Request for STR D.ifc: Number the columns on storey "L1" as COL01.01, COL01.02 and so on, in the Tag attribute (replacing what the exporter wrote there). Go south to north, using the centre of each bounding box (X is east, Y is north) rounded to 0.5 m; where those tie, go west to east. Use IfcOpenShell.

First a look at what the model holds.

```python
import ifcopenshell
import ifcopenshell.util.element
import ifcopenshell.util.placement

model = ifcopenshell.open("STR D.ifc")
print(model.schema)
storey = next(s for s in model.by_type("IfcBuildingStorey") if s.Name == "L1")
columns = [e for e in ifcopenshell.util.element.get_decomposition(storey) if e.is_a("IfcColumn")]
for e in sorted(columns, key=lambda e: e.id()):
    origin = ifcopenshell.util.placement.get_local_placement(e.ObjectPlacement)[:3, 3]
    print(e.id(), e.Tag, e.Name, origin.round(2) + 0.0, sep=" | ")
```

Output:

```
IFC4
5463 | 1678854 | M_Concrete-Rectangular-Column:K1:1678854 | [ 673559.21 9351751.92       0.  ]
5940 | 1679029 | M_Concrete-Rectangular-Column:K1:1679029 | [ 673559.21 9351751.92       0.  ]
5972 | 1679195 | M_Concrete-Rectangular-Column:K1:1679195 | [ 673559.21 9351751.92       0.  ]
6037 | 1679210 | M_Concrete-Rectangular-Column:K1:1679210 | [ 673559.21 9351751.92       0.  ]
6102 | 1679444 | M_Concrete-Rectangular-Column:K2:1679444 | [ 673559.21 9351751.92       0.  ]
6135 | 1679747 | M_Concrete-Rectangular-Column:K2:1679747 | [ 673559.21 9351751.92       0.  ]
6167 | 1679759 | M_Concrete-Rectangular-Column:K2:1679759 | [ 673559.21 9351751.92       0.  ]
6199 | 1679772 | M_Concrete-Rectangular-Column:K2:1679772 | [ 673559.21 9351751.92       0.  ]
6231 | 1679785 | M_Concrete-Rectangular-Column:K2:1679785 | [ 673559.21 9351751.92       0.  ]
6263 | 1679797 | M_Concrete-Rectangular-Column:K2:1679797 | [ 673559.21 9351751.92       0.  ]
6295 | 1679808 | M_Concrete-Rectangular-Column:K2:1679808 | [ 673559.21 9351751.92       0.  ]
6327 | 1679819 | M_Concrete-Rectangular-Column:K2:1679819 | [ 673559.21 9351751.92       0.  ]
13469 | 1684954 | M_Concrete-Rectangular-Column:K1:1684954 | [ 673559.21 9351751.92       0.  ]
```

```python
import ifcopenshell
import ifcopenshell.geom
import ifcopenshell.util.element
import ifcopenshell.util.shape

model = ifcopenshell.open("STR D.ifc")
settings = ifcopenshell.geom.settings()
settings.set("use-world-coords", True)


def centre(element):
    shape = ifcopenshell.geom.create_shape(settings, element)
    return ifcopenshell.util.shape.get_bbox_centroid(shape.geometry)


storey = next(s for s in model.by_type("IfcBuildingStorey") if s.Name == "L1")
columns = [e for e in ifcopenshell.util.element.get_decomposition(storey) if e.is_a("IfcColumn")]

# Insertion points can sit at a corner or the storey origin, so sort by the geometry (in metres).
centres = {e: centre(e) for e in columns}
columns.sort(key=lambda e: (round(centres[e][1] / 0.5), centres[e][0]))

for i, e in enumerate(columns, start=1):
    number = f"COL01.{i:02d}"
    e.Tag = number
    print(e.id(), number)

model.write("STR D_edited.ifc")
```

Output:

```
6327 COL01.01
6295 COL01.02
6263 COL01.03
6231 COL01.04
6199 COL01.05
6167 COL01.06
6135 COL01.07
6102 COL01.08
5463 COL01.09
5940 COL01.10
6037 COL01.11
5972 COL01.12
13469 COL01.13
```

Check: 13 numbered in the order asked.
